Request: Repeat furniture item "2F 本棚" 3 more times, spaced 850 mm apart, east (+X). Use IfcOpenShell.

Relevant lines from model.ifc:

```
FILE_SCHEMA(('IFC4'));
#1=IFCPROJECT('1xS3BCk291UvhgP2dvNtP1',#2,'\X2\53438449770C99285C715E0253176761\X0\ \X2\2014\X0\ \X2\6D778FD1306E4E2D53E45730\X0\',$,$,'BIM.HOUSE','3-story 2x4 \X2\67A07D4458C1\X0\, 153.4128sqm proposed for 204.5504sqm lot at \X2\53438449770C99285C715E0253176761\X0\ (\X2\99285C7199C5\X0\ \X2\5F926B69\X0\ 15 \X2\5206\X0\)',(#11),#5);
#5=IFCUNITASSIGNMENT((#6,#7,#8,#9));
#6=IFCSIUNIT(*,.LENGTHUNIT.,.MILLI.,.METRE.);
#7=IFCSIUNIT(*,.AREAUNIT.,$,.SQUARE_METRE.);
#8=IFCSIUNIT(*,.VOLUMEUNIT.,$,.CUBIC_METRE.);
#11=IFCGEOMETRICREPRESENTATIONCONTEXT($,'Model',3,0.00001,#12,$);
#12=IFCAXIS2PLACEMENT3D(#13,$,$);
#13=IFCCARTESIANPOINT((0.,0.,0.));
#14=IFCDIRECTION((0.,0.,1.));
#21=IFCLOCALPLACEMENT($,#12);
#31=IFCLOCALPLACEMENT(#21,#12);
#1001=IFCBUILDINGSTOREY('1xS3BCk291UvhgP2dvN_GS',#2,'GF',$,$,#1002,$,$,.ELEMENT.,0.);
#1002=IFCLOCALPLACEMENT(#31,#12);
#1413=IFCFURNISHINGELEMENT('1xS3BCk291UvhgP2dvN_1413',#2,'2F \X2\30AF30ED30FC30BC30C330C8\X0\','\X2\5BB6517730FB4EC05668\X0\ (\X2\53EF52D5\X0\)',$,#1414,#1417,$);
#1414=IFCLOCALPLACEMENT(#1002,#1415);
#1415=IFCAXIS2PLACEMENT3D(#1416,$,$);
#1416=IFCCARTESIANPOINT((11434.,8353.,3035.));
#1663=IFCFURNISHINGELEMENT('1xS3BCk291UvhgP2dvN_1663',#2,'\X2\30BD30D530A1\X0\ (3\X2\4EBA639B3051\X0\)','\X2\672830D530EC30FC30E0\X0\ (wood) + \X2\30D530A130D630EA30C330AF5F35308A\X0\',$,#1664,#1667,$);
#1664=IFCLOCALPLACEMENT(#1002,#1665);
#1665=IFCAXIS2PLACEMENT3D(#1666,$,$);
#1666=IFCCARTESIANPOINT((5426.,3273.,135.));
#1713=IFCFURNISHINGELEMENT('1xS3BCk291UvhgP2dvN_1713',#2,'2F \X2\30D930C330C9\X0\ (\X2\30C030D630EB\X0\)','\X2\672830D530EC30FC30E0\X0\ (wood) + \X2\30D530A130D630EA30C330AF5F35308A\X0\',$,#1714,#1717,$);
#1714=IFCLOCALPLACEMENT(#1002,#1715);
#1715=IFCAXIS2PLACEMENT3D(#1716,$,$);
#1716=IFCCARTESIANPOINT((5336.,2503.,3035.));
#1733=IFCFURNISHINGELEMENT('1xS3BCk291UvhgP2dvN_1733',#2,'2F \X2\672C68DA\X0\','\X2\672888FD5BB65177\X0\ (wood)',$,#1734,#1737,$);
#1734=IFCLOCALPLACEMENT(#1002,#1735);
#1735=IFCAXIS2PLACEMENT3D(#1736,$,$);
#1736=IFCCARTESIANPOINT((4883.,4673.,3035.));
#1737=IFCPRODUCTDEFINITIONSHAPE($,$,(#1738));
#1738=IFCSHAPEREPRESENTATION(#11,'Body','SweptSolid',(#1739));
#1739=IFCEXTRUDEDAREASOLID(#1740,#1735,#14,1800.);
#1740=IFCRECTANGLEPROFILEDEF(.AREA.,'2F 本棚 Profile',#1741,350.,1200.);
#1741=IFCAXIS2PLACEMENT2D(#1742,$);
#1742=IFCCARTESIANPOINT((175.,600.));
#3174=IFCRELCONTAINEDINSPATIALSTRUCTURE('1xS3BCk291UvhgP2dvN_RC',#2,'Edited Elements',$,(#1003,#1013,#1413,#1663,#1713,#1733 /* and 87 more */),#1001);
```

```python
import numpy as np
import ifcopenshell
import ifcopenshell.api.geometry
import ifcopenshell.api.root
import ifcopenshell.util.element
import ifcopenshell.util.placement

model = ifcopenshell.open("model.ifc")


def reuse_history(source, copy):
    """copy_class also copies each property set's owner history, people and application; keep the originals."""
    for rel in copy.IsDefinedBy:
        if rel.is_a("IfcRelDefinesByProperties") and (history := rel.RelatingPropertyDefinition.OwnerHistory):
            rel.RelatingPropertyDefinition.OwnerHistory = source.OwnerHistory
            ifcopenshell.util.element.remove_deep2(model, history)


source = model.by_guid("1xS3BCk291UvhgP2dvN_1733")
base = ifcopenshell.util.placement.get_local_placement(source.ObjectPlacement)
step = np.array([1.0, 0.0, 0.0]) * 850.0

for i in range(1, 4):
    copy = ifcopenshell.api.root.copy_class(model, product=source)
    copy.Representation = ifcopenshell.util.element.copy_deep(
        model, source.Representation, exclude=["IfcGeometricRepresentationContext", "IfcRepresentationMap"]
    )
    reuse_history(source, copy)
    matrix = base.copy()
    matrix[:3, 3] += i * step
    print("added at", matrix[:3, 3].round(3) + 0.0)
    ifcopenshell.api.geometry.edit_object_placement(model, product=copy, matrix=matrix, is_si=False)

model.write("model_edited.ifc")
```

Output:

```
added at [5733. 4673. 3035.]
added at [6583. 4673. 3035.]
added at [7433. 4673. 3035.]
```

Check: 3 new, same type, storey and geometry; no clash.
